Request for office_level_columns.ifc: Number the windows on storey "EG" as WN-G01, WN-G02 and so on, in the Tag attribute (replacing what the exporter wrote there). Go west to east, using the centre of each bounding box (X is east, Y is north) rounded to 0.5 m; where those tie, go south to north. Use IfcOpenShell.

First a look at what the model holds.

```python
import ifcopenshell
import ifcopenshell.util.element
import ifcopenshell.util.placement

model = ifcopenshell.open("office_level_columns.ifc")
print(model.schema)
storey = next(s for s in model.by_type("IfcBuildingStorey") if s.Name == "EG")
windows = [e for e in ifcopenshell.util.element.get_decomposition(storey) if e.is_a("IfcWindow")]
for e in sorted(windows, key=lambda e: e.id()):
    origin = ifcopenshell.util.placement.get_local_placement(e.ObjectPlacement)[:3, 3]
    print(e.id(), e.Tag, e.Name, origin.round(2) + 0.0, sep=" | ")
```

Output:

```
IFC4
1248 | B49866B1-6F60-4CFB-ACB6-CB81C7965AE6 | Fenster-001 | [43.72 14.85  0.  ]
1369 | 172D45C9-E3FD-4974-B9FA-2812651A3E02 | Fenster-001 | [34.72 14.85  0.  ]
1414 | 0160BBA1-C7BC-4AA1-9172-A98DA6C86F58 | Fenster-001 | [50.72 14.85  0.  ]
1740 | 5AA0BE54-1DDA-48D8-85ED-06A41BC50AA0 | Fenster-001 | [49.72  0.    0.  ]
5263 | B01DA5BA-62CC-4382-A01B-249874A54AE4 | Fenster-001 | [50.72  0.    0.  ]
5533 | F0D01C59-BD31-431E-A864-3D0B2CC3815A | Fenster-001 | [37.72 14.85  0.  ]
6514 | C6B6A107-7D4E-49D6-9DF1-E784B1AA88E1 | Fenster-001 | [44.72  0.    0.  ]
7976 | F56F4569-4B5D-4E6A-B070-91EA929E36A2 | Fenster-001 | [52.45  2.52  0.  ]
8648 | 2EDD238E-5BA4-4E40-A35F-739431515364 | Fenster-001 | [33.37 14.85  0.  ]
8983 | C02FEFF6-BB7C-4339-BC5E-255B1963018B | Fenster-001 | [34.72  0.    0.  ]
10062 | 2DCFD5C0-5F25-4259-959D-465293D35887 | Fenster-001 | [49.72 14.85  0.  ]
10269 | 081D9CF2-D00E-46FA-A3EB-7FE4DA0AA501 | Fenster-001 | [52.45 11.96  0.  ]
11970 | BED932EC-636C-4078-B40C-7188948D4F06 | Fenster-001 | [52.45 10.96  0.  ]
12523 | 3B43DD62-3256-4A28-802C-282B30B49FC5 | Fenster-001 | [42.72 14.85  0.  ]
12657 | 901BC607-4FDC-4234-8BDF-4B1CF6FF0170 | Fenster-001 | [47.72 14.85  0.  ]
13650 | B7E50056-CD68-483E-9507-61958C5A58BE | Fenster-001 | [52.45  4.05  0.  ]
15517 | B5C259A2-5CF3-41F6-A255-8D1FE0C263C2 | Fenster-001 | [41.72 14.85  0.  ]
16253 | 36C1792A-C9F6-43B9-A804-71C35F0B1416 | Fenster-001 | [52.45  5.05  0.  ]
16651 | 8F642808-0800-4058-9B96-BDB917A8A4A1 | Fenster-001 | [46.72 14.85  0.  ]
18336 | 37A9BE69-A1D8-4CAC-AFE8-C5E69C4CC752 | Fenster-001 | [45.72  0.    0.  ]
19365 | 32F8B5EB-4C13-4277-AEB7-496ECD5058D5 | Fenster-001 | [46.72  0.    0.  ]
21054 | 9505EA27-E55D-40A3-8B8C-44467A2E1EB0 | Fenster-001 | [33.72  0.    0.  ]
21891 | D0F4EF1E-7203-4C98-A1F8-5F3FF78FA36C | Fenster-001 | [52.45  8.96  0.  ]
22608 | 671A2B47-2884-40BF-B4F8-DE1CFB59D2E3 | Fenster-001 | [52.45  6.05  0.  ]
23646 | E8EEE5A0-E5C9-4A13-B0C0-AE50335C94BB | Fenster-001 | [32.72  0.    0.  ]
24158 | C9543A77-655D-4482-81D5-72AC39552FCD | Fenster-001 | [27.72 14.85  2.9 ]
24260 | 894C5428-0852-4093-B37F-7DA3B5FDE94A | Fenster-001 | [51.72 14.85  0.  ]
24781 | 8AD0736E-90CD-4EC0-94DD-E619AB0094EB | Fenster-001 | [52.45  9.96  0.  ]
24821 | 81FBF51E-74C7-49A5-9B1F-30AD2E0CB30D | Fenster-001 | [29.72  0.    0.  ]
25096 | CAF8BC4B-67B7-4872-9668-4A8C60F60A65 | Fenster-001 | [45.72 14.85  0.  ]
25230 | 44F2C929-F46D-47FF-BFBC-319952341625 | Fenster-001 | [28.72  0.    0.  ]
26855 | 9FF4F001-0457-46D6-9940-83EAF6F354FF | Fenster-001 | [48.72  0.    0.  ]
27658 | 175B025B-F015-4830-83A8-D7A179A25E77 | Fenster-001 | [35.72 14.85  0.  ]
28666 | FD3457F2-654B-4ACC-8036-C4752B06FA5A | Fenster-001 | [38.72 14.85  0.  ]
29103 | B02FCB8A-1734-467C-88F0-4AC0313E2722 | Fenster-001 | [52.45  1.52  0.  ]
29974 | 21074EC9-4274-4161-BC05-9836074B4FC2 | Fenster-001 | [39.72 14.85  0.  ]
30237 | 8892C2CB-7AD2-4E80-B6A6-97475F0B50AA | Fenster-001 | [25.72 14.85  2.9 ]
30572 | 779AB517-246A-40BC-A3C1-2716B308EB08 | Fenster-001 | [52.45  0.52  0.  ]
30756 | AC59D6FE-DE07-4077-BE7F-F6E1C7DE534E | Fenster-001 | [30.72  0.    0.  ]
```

```python
import ifcopenshell
import ifcopenshell.geom
import ifcopenshell.util.element
import ifcopenshell.util.shape

model = ifcopenshell.open("office_level_columns.ifc")
settings = ifcopenshell.geom.settings()
settings.set("use-world-coords", True)


def centre(element):
    shape = ifcopenshell.geom.create_shape(settings, element)
    return ifcopenshell.util.shape.get_bbox_centroid(shape.geometry)


storey = next(s for s in model.by_type("IfcBuildingStorey") if s.Name == "EG")
windows = [e for e in ifcopenshell.util.element.get_decomposition(storey) if e.is_a("IfcWindow")]

# Insertion points can sit at a corner or the storey origin, so sort by the geometry (in metres).
centres = {e: centre(e) for e in windows}
windows.sort(key=lambda e: (round(centres[e][0] / 0.5), centres[e][1]))

for i, e in enumerate(windows, start=1):
    number = f"WN-G{i:02d}"
    e.Tag = number
    print(e.id(), number)

model.write("office_level_columns-out.ifc")
```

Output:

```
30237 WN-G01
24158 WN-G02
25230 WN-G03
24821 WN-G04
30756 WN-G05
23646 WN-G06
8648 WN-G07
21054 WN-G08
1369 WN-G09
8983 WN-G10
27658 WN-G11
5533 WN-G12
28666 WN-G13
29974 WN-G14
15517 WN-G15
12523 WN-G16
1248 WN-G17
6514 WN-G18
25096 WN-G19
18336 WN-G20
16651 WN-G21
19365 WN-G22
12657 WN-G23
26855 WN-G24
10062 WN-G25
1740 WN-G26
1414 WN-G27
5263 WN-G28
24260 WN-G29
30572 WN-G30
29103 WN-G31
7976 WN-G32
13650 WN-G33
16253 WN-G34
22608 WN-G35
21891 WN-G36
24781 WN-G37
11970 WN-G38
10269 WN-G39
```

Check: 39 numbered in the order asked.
